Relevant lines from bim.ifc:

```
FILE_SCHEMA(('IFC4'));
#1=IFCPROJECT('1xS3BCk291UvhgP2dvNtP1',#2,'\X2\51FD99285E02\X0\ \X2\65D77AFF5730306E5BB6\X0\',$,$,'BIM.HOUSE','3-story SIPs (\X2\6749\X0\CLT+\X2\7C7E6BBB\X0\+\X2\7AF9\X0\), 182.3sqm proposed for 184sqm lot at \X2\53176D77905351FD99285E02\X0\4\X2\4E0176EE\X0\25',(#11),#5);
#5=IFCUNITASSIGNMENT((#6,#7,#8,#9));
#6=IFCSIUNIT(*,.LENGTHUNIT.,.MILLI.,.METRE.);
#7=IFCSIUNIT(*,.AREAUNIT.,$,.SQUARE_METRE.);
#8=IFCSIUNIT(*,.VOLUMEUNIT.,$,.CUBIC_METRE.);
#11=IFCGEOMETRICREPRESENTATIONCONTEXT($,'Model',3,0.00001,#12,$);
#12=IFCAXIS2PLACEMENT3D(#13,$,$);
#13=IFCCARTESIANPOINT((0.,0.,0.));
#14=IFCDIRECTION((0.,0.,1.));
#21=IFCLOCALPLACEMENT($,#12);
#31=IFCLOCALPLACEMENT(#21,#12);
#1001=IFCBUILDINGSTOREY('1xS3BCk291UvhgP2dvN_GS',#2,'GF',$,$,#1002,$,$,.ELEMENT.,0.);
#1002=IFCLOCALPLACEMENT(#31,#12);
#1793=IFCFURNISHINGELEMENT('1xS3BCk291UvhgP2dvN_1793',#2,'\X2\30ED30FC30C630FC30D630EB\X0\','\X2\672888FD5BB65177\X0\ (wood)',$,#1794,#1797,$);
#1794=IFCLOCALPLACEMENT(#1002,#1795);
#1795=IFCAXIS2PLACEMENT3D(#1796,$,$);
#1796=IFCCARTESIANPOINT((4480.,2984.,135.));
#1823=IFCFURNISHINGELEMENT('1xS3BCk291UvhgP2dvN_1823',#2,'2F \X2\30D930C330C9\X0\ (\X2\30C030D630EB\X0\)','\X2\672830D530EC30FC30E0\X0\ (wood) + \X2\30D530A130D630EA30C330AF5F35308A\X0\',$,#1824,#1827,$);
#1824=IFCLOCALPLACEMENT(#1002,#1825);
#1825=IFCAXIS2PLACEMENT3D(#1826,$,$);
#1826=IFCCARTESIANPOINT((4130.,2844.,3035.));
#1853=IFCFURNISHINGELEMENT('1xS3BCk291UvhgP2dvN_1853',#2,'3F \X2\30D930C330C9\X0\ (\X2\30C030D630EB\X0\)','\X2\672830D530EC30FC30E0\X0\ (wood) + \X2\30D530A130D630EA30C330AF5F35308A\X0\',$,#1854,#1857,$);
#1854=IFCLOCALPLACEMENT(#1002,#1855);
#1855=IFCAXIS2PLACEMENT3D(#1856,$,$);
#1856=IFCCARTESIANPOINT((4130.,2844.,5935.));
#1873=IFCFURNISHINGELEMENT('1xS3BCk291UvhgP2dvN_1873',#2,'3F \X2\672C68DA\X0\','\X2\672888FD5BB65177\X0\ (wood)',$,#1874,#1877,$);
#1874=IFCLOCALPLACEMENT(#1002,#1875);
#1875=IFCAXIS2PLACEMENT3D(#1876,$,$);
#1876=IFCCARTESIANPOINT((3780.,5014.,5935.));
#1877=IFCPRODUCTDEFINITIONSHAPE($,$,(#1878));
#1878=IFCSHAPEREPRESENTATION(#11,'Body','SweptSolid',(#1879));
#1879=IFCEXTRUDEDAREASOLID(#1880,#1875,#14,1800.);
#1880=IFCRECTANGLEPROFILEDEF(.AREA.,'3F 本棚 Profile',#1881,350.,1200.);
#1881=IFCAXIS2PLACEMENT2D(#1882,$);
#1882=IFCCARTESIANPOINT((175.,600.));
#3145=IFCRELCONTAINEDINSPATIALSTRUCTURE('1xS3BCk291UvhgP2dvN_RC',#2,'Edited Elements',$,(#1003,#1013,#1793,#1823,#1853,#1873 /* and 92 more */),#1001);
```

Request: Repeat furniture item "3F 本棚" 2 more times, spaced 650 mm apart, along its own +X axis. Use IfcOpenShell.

```python
import ifcopenshell
import ifcopenshell.api.geometry
import ifcopenshell.api.root
import ifcopenshell.util.element
import ifcopenshell.util.placement
import ifcopenshell.util.unit

model = ifcopenshell.open("bim.ifc")
unit_scale = ifcopenshell.util.unit.calculate_unit_scale(model)


def reuse_history(source, copy):
    """copy_class also copies each property set's owner history, people and application; keep the originals."""
    for rel in copy.IsDefinedBy:
        if rel.is_a("IfcRelDefinesByProperties") and (history := rel.RelatingPropertyDefinition.OwnerHistory):
            rel.RelatingPropertyDefinition.OwnerHistory = source.OwnerHistory
            ifcopenshell.util.element.remove_deep2(model, history)


source = model.by_id(1873)
base = ifcopenshell.util.placement.get_local_placement(source.ObjectPlacement)
step = base[:3, 0] * 0.65 / unit_scale

for i in range(1, 3):
    copy = ifcopenshell.api.root.copy_class(model, product=source)
    copy.Representation = ifcopenshell.util.element.copy_deep(
        model, source.Representation, exclude=["IfcGeometricRepresentationContext", "IfcRepresentationMap"]
    )
    reuse_history(source, copy)
    matrix = base.copy()
    matrix[:3, 3] += i * step
    print("added at", matrix[:3, 3].round(3) + 0.0)
    ifcopenshell.api.geometry.edit_object_placement(model, product=copy, matrix=matrix, is_si=False)

model.write("bim_v2.ifc")
```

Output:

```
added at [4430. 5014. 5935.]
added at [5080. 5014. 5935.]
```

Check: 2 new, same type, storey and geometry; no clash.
